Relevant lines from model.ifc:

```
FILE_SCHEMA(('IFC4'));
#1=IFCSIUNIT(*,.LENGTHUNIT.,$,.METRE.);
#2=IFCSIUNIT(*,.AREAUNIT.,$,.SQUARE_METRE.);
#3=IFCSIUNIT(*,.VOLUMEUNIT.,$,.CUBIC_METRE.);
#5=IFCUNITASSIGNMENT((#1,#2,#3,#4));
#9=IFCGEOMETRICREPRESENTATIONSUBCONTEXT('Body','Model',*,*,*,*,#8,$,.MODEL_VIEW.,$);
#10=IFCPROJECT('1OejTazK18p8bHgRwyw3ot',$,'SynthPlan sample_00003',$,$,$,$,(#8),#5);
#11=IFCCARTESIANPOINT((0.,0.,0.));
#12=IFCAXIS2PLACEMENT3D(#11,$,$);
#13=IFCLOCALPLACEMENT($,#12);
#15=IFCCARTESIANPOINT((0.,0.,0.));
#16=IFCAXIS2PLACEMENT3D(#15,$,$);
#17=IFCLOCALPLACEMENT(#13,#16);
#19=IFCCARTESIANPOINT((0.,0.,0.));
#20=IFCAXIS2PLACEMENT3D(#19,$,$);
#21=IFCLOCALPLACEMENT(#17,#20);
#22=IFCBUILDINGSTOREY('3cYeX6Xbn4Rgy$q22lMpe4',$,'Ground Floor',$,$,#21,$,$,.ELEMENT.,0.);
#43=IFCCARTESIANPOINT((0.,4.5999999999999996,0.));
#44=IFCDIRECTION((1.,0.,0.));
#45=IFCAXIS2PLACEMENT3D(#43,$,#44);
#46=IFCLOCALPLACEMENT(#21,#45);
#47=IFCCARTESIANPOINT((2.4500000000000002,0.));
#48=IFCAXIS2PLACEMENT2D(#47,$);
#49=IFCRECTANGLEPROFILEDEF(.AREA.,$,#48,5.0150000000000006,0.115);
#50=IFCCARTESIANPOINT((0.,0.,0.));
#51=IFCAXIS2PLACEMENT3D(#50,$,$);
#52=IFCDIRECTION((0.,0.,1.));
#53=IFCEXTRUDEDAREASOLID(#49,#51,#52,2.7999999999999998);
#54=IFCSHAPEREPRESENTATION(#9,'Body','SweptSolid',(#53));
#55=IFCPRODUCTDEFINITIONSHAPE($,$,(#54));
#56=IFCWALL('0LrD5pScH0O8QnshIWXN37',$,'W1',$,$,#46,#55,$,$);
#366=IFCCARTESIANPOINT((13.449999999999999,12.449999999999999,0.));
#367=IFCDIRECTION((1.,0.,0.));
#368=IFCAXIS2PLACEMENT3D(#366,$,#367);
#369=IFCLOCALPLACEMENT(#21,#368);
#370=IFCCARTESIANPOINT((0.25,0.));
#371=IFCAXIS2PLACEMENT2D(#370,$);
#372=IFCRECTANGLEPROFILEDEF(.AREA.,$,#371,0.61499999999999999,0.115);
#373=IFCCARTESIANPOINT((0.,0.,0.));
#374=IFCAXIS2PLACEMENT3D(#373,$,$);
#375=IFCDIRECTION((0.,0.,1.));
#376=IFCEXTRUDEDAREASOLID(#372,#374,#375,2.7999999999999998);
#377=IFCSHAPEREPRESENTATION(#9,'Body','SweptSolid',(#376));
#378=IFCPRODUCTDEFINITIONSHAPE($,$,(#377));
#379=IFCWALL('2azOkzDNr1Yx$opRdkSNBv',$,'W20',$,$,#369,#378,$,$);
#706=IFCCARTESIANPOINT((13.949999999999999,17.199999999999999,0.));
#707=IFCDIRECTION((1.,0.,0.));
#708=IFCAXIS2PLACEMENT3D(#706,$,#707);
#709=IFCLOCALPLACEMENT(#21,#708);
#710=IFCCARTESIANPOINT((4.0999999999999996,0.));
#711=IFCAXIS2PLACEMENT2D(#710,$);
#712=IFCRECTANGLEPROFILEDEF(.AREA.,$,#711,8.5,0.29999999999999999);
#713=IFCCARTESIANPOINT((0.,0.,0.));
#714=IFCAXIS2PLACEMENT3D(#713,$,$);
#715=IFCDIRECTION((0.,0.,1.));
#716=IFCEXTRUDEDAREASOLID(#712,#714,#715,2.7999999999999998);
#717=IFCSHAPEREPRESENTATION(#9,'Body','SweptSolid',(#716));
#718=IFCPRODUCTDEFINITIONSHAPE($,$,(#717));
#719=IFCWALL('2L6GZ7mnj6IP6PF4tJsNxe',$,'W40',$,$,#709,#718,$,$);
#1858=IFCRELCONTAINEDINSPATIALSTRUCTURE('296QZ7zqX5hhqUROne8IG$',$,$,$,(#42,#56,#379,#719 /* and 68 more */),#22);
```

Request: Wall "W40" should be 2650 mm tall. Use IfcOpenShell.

```python
import ifcopenshell
import ifcopenshell.geom
import ifcopenshell.util.representation
import ifcopenshell.util.shape
import ifcopenshell.util.unit

model = ifcopenshell.open("model.ifc")
unit_scale = ifcopenshell.util.unit.calculate_unit_scale(model)
settings = ifcopenshell.geom.settings()


def volume(element):
    """Net volume in cubic metres, openings subtracted."""
    shape = ifcopenshell.geom.create_shape(settings, element)
    return ifcopenshell.util.shape.get_volume(shape.geometry)


wall = model.by_id(719)
before = volume(wall)

body = ifcopenshell.util.representation.get_representation(wall, "Model", "Body")
solid = body.Items[0]
old_height = solid.Depth
solid.Depth = 2.65 / unit_scale
after = volume(wall)

print(f"height {old_height:g} -> {solid.Depth:g}, volume {before:.3f} -> {after:.3f} m3")

model.write("model-out.ifc")
```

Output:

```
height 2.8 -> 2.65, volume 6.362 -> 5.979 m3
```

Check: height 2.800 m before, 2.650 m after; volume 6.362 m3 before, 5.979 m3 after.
